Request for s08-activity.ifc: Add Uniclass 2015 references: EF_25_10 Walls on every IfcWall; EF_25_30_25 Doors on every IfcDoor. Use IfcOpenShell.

First a look at what the model holds.

```python
import ifcopenshell

model = ifcopenshell.open("s08-activity.ifc")
print(model.schema)
print("classifications:", [c.Name for c in model.by_type("IfcClassification")])
for ifc_class in ("IfcDoor", "IfcRoof", "IfcStair", "IfcWall", "IfcWindow"):
    print(ifc_class, len(model.by_type(ifc_class)))
```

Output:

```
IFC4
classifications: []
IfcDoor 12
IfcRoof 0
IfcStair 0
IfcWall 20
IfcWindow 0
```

```python
import ifcopenshell
import ifcopenshell.api.classification

model = ifcopenshell.open("s08-activity.ifc")

system = ifcopenshell.api.classification.add_classification(model, classification="Uniclass 2015")

codes = {
    "IfcWall": ("EF_25_10", "Walls"),
    "IfcDoor": ("EF_25_30_25", "Doors"),
}
for ifc_class, (code, name) in codes.items():
    products = model.by_type(ifc_class)
    ifcopenshell.api.classification.add_reference(
        model, products=products, classification=system, identification=code, name=name
    )
    print(code, len(products))

model.write("s08-activity_edited.ifc")
```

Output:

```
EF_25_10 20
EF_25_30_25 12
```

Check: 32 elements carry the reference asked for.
